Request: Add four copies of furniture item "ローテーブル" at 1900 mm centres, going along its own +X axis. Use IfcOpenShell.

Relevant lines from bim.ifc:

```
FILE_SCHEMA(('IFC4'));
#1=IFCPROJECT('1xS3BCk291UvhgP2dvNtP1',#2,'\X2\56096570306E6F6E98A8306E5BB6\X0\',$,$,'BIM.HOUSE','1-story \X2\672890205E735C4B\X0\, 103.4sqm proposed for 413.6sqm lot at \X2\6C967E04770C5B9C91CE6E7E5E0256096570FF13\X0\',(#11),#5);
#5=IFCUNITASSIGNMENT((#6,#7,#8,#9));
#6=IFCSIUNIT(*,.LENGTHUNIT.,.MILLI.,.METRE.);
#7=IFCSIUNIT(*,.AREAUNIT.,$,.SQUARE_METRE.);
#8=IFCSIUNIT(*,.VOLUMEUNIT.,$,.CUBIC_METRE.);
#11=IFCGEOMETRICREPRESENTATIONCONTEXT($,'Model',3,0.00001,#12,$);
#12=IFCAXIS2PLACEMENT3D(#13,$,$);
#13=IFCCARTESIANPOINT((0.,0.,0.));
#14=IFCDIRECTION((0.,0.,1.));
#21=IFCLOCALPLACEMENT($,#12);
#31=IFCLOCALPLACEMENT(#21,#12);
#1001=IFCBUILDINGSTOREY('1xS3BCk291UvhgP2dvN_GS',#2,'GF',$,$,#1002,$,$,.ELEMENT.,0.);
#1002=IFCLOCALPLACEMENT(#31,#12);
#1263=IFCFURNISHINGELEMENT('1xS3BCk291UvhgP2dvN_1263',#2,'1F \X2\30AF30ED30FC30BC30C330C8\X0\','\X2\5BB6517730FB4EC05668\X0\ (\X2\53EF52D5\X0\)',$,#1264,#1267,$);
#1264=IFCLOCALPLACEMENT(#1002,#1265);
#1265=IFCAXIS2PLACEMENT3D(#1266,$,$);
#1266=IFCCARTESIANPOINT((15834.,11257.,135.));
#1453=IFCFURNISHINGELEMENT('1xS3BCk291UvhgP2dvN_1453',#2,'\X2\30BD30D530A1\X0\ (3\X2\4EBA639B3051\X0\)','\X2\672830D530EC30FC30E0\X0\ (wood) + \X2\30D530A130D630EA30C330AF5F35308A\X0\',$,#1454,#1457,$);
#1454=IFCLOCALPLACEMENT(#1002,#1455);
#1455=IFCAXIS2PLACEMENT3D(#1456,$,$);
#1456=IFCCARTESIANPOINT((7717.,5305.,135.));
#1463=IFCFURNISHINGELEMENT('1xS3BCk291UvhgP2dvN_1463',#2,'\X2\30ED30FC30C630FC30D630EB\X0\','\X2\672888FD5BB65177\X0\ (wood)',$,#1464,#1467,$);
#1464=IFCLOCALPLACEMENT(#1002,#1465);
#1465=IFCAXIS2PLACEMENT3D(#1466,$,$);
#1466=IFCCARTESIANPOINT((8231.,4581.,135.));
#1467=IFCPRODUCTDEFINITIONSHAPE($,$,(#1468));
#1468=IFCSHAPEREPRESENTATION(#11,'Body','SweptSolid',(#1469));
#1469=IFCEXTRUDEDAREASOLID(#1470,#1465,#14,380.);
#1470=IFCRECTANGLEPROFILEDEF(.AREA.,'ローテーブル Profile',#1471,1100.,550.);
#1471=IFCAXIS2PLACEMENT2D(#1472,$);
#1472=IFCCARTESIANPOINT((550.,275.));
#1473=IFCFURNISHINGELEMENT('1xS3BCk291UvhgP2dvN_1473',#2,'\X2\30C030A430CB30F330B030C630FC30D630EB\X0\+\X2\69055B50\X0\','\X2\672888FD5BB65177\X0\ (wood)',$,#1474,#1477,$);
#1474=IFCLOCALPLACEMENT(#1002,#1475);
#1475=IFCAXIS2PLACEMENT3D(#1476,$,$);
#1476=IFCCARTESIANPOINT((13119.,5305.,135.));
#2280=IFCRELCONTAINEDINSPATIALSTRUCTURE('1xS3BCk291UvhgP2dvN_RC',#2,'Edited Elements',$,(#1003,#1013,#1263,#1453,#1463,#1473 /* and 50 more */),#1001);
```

```python
import ifcopenshell
import ifcopenshell.api.geometry
import ifcopenshell.api.root
import ifcopenshell.util.element
import ifcopenshell.util.placement
import ifcopenshell.util.unit

model = ifcopenshell.open("bim.ifc")
unit_scale = ifcopenshell.util.unit.calculate_unit_scale(model)


def reuse_history(source, copy):
    """copy_class also copies each property set's owner history, people and application; keep the originals."""
    for rel in copy.IsDefinedBy:
        if rel.is_a("IfcRelDefinesByProperties") and (history := rel.RelatingPropertyDefinition.OwnerHistory):
            rel.RelatingPropertyDefinition.OwnerHistory = source.OwnerHistory
            ifcopenshell.util.element.remove_deep2(model, history)


source = model.by_guid("1xS3BCk291UvhgP2dvN_1463")
base = ifcopenshell.util.placement.get_local_placement(source.ObjectPlacement)
step = base[:3, 0] * 1.9 / unit_scale

for i in range(1, 5):
    copy = ifcopenshell.api.root.copy_class(model, product=source)
    copy.Representation = ifcopenshell.util.element.copy_deep(
        model, source.Representation, exclude=["IfcGeometricRepresentationContext", "IfcRepresentationMap"]
    )
    reuse_history(source, copy)
    matrix = base.copy()
    matrix[:3, 3] += i * step
    print("added at", matrix[:3, 3].round(3) + 0.0)
    ifcopenshell.api.geometry.edit_object_placement(model, product=copy, matrix=matrix, is_si=False)

model.write("bim-out.ifc")
```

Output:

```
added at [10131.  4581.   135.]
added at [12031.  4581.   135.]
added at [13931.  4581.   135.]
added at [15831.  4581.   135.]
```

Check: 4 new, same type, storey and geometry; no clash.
